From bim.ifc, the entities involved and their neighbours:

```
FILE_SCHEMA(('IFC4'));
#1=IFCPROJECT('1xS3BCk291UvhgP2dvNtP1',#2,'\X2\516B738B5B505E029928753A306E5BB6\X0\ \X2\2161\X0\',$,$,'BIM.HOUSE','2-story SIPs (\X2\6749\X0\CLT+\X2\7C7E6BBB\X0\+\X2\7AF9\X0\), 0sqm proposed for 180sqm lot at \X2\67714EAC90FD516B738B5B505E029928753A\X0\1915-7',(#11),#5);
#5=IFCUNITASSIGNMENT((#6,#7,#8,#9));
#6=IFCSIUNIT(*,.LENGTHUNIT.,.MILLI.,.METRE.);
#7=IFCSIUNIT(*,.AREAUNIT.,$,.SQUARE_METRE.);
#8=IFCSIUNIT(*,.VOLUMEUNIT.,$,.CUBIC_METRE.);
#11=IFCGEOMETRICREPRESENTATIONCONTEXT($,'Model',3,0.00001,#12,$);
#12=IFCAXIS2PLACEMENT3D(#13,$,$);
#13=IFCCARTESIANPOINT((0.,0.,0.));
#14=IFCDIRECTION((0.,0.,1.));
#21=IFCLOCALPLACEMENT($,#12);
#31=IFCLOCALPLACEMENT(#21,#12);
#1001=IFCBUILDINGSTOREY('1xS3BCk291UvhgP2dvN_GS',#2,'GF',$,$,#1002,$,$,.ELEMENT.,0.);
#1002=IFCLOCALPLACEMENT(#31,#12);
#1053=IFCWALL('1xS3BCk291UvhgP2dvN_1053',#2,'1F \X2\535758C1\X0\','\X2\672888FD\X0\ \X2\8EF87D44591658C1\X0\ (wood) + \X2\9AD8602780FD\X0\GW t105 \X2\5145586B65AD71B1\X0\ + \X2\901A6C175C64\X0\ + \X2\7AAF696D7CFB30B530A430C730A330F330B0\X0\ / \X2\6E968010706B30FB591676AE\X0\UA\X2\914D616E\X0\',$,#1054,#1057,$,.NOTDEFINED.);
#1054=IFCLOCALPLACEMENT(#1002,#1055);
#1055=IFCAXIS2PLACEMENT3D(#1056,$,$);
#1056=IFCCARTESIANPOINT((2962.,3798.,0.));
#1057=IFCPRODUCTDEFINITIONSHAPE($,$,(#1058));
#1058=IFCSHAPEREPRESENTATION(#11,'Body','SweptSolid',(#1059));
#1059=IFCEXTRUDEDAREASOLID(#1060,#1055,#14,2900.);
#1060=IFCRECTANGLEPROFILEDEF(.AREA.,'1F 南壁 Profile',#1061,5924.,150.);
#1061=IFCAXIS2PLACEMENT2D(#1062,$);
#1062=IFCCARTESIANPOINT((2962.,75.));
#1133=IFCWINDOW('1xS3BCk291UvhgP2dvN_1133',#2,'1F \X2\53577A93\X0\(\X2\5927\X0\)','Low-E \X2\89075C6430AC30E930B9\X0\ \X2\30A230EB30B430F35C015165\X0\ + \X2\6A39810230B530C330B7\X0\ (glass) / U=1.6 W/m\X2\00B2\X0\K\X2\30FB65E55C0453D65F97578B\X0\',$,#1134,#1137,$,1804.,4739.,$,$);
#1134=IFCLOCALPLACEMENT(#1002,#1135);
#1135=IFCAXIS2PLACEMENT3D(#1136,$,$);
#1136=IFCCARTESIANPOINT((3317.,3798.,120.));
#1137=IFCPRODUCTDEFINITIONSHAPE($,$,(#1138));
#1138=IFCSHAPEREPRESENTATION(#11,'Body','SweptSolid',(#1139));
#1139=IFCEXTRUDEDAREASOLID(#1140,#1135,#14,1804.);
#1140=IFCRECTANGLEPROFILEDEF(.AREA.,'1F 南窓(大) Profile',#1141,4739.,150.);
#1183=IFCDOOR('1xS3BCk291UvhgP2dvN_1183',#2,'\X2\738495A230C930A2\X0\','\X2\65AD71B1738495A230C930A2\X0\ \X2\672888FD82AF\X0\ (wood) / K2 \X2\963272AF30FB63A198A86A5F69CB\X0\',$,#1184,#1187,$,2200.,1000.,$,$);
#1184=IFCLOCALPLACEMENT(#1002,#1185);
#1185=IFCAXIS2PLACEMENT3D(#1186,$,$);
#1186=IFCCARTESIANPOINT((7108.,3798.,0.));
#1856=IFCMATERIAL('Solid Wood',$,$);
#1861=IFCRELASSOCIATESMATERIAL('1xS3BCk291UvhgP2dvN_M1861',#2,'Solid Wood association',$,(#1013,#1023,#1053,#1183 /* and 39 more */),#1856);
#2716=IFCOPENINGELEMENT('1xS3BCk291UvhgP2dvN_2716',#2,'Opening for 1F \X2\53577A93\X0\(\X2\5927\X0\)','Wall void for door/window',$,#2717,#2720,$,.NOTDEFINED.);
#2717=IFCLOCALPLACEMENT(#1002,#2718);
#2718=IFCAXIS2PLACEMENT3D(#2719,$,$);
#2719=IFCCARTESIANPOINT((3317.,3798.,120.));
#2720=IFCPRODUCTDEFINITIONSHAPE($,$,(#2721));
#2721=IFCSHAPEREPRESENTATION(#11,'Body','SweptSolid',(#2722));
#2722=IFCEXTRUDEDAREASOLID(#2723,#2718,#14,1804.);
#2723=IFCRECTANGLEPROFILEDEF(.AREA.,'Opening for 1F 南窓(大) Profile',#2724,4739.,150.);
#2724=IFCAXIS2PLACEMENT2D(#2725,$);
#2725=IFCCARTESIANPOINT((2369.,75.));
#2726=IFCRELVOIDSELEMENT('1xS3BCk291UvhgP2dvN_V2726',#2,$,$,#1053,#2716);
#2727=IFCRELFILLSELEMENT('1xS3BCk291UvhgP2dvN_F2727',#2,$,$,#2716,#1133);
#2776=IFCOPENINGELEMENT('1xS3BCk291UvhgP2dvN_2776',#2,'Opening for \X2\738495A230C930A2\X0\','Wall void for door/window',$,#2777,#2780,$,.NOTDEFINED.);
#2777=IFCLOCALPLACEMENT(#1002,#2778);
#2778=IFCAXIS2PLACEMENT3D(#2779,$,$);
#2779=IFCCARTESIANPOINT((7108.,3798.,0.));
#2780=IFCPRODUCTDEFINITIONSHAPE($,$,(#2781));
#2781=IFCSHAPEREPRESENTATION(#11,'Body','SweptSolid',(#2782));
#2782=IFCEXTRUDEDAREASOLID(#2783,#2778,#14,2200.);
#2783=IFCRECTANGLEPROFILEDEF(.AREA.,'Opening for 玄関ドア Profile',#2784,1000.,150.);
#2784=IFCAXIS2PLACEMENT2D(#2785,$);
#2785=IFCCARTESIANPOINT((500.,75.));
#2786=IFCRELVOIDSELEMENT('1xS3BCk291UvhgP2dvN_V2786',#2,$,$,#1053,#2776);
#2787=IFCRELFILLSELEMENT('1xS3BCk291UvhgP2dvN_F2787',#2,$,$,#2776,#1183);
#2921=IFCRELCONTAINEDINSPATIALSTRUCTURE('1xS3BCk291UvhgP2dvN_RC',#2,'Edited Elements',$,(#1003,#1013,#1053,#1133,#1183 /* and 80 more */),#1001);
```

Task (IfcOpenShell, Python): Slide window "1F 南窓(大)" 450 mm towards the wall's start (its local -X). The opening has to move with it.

```python
import ifcopenshell
import ifcopenshell.api.geometry
import ifcopenshell.util.placement
import ifcopenshell.util.unit

model = ifcopenshell.open("bim.ifc")
unit_scale = ifcopenshell.util.unit.calculate_unit_scale(model)

window = model.by_guid("1xS3BCk291UvhgP2dvN_1133")
opening = window.FillsVoids[0].RelatingOpeningElement
wall = opening.VoidsElements[0].RelatingBuildingElement

wall_matrix = ifcopenshell.util.placement.get_local_placement(wall.ObjectPlacement)
shift = wall_matrix[:3, 0] * -0.45 / unit_scale
before = ifcopenshell.util.placement.get_local_placement(window.ObjectPlacement)[:3, 3].copy()

# The window is not placed relative to its opening, so move both.
for product in (opening, window):
    matrix = ifcopenshell.util.placement.get_local_placement(product.ObjectPlacement)
    matrix[:3, 3] += shift
    ifcopenshell.api.geometry.edit_object_placement(model, product=product, matrix=matrix, is_si=False)

after = ifcopenshell.util.placement.get_local_placement(window.ObjectPlacement)[:3, 3]
print("window moved by", (after - before).round(3) + 0.0)

model.write("bim_updated.ifc")
```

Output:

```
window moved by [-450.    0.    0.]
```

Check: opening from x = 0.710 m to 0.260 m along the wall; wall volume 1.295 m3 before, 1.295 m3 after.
